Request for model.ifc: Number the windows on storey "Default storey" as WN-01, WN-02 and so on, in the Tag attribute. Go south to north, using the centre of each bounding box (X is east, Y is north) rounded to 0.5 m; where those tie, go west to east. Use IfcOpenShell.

First a look at what the model holds.

```python
import ifcopenshell
import ifcopenshell.util.element
import ifcopenshell.util.placement

model = ifcopenshell.open("model.ifc")
print(model.schema)
storey = next(s for s in model.by_type("IfcBuildingStorey") if s.Name == "Default storey")
windows = [e for e in ifcopenshell.util.element.get_decomposition(storey) if e.is_a("IfcWindow")]
for e in sorted(windows, key=lambda e: e.id()):
    origin = ifcopenshell.util.placement.get_local_placement(e.ObjectPlacement)[:3, 3]
    print(e.id(), e.Tag, e.Name, origin.round(2) + 0.0, sep=" | ")
```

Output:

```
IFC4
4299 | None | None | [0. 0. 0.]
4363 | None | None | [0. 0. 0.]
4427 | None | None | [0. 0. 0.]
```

```python
import ifcopenshell
import ifcopenshell.geom
import ifcopenshell.util.element
import ifcopenshell.util.shape

model = ifcopenshell.open("model.ifc")
settings = ifcopenshell.geom.settings()
settings.set("use-world-coords", True)


def centre(element):
    shape = ifcopenshell.geom.create_shape(settings, element)
    return ifcopenshell.util.shape.get_bbox_centroid(shape.geometry)


storey = next(s for s in model.by_type("IfcBuildingStorey") if s.Name == "Default storey")
windows = [e for e in ifcopenshell.util.element.get_decomposition(storey) if e.is_a("IfcWindow")]

# Insertion points can sit at a corner or the storey origin, so sort by the geometry (in metres).
centres = {e: centre(e) for e in windows}
windows.sort(key=lambda e: (round(centres[e][1] / 0.5), centres[e][0]))

for i, e in enumerate(windows, start=1):
    number = f"WN-{i:02d}"
    e.Tag = number
    print(e.id(), number)

model.write("model_v2.ifc")
```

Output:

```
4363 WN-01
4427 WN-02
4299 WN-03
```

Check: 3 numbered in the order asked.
